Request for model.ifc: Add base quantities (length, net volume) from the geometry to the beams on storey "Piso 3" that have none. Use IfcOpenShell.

First a look at what the model holds.

```python
import ifcopenshell
import ifcopenshell.util.element
import ifcopenshell.util.unit

model = ifcopenshell.open("model.ifc")
print(model.schema)
for unit_type in ("LENGTHUNIT", "AREAUNIT", "VOLUMEUNIT"):
    print(unit_type, ifcopenshell.util.unit.calculate_unit_scale(model, unit_type))
storey = next(s for s in model.by_type("IfcBuildingStorey") if s.Name == "Piso 3")
beams = [e for e in ifcopenshell.util.element.get_decomposition(storey) if e.is_a("IfcBeam")]
for e in sorted(beams, key=lambda e: e.id()):
    print(e.id(), e.is_a(), e.Name, list(ifcopenshell.util.element.get_psets(e, qtos_only=True)), sep=" | ")
```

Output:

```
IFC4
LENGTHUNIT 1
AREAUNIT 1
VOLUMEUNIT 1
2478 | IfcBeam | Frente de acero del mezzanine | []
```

```python
import ifcopenshell
import ifcopenshell.api.pset
import ifcopenshell.geom
import ifcopenshell.util.element
import ifcopenshell.util.shape
import ifcopenshell.util.unit

model = ifcopenshell.open("model.ifc")
unit_scale = ifcopenshell.util.unit.calculate_unit_scale(model)
volume_scale = ifcopenshell.util.unit.calculate_unit_scale(model, "VOLUMEUNIT")
settings = ifcopenshell.geom.settings()

storey = next(s for s in model.by_type("IfcBuildingStorey") if s.Name == "Piso 3")
beams = [e for e in ifcopenshell.util.element.get_decomposition(storey) if e.is_a("IfcBeam")]

for e in sorted(beams, key=lambda e: e.id()):
    if ifcopenshell.util.element.get_psets(e, qtos_only=True, should_inherit=False):
        continue
    # Geometry comes back in metres, in the element's own axes.
    shape = ifcopenshell.geom.create_shape(settings, e)
    values = {
        "Length": ifcopenshell.util.shape.get_max_xyz(shape.geometry) / unit_scale,
        "NetVolume": ifcopenshell.util.shape.get_volume(shape.geometry) / volume_scale,
    }
    qto = ifcopenshell.api.pset.add_qto(model, product=e, name="Qto_BeamBaseQuantities")
    ifcopenshell.api.pset.edit_qto(model, qto=qto, properties=values)
    print(e.id(), {k: round(v, 3) for k, v in values.items()})

model.write("model_v2.ifc")
```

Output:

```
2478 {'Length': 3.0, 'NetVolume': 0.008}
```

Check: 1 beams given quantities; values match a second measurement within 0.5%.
